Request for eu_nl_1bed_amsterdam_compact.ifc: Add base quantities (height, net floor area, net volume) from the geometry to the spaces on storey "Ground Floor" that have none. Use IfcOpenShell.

First a look at what the model holds.

```python
import ifcopenshell
import ifcopenshell.util.element
import ifcopenshell.util.unit

model = ifcopenshell.open("eu_nl_1bed_amsterdam_compact.ifc")
print(model.schema)
for unit_type in ("LENGTHUNIT", "AREAUNIT", "VOLUMEUNIT"):
    print(unit_type, ifcopenshell.util.unit.calculate_unit_scale(model, unit_type))
storey = next(s for s in model.by_type("IfcBuildingStorey") if s.Name == "Ground Floor")
spaces = [e for e in ifcopenshell.util.element.get_decomposition(storey) if e.is_a("IfcSpace")]
for e in sorted(spaces, key=lambda e: e.id()):
    print(e.id(), e.is_a(), e.Name, list(ifcopenshell.util.element.get_psets(e, qtos_only=True)), sep=" | ")
```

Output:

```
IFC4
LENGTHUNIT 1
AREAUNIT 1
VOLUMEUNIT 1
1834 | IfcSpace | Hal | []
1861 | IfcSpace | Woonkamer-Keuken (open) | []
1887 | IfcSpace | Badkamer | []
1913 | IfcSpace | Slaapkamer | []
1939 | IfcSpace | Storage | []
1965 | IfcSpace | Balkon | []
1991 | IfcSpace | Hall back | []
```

```python
import ifcopenshell
import ifcopenshell.api.pset
import ifcopenshell.geom
import ifcopenshell.util.element
import ifcopenshell.util.shape
import ifcopenshell.util.unit

model = ifcopenshell.open("eu_nl_1bed_amsterdam_compact.ifc")
unit_scale = ifcopenshell.util.unit.calculate_unit_scale(model)
area_scale = ifcopenshell.util.unit.calculate_unit_scale(model, "AREAUNIT")
volume_scale = ifcopenshell.util.unit.calculate_unit_scale(model, "VOLUMEUNIT")
settings = ifcopenshell.geom.settings()

storey = next(s for s in model.by_type("IfcBuildingStorey") if s.Name == "Ground Floor")
spaces = [e for e in ifcopenshell.util.element.get_decomposition(storey) if e.is_a("IfcSpace")]

for e in sorted(spaces, key=lambda e: e.id()):
    if ifcopenshell.util.element.get_psets(e, qtos_only=True, should_inherit=False):
        continue
    # Geometry comes back in metres, in the element's own axes.
    shape = ifcopenshell.geom.create_shape(settings, e)
    values = {
        "Height": ifcopenshell.util.shape.get_z(shape.geometry) / unit_scale,
        "NetFloorArea": ifcopenshell.util.shape.get_footprint_area(shape.geometry) / area_scale,
        "NetVolume": ifcopenshell.util.shape.get_volume(shape.geometry) / volume_scale,
    }
    qto = ifcopenshell.api.pset.add_qto(model, product=e, name="Qto_SpaceBaseQuantities")
    ifcopenshell.api.pset.edit_qto(model, qto=qto, properties=values)
    print(e.id(), {k: round(v, 3) for k, v in values.items()})

model.write("eu_nl_1bed_amsterdam_compact-out.ifc")
```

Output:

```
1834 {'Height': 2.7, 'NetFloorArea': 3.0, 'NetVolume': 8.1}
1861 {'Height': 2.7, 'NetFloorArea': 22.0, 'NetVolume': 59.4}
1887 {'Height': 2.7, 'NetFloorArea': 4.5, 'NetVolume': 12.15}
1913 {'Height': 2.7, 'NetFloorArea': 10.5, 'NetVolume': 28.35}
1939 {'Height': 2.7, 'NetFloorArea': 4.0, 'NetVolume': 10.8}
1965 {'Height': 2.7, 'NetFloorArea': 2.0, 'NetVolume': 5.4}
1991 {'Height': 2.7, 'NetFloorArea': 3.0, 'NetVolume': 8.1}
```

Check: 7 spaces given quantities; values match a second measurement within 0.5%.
